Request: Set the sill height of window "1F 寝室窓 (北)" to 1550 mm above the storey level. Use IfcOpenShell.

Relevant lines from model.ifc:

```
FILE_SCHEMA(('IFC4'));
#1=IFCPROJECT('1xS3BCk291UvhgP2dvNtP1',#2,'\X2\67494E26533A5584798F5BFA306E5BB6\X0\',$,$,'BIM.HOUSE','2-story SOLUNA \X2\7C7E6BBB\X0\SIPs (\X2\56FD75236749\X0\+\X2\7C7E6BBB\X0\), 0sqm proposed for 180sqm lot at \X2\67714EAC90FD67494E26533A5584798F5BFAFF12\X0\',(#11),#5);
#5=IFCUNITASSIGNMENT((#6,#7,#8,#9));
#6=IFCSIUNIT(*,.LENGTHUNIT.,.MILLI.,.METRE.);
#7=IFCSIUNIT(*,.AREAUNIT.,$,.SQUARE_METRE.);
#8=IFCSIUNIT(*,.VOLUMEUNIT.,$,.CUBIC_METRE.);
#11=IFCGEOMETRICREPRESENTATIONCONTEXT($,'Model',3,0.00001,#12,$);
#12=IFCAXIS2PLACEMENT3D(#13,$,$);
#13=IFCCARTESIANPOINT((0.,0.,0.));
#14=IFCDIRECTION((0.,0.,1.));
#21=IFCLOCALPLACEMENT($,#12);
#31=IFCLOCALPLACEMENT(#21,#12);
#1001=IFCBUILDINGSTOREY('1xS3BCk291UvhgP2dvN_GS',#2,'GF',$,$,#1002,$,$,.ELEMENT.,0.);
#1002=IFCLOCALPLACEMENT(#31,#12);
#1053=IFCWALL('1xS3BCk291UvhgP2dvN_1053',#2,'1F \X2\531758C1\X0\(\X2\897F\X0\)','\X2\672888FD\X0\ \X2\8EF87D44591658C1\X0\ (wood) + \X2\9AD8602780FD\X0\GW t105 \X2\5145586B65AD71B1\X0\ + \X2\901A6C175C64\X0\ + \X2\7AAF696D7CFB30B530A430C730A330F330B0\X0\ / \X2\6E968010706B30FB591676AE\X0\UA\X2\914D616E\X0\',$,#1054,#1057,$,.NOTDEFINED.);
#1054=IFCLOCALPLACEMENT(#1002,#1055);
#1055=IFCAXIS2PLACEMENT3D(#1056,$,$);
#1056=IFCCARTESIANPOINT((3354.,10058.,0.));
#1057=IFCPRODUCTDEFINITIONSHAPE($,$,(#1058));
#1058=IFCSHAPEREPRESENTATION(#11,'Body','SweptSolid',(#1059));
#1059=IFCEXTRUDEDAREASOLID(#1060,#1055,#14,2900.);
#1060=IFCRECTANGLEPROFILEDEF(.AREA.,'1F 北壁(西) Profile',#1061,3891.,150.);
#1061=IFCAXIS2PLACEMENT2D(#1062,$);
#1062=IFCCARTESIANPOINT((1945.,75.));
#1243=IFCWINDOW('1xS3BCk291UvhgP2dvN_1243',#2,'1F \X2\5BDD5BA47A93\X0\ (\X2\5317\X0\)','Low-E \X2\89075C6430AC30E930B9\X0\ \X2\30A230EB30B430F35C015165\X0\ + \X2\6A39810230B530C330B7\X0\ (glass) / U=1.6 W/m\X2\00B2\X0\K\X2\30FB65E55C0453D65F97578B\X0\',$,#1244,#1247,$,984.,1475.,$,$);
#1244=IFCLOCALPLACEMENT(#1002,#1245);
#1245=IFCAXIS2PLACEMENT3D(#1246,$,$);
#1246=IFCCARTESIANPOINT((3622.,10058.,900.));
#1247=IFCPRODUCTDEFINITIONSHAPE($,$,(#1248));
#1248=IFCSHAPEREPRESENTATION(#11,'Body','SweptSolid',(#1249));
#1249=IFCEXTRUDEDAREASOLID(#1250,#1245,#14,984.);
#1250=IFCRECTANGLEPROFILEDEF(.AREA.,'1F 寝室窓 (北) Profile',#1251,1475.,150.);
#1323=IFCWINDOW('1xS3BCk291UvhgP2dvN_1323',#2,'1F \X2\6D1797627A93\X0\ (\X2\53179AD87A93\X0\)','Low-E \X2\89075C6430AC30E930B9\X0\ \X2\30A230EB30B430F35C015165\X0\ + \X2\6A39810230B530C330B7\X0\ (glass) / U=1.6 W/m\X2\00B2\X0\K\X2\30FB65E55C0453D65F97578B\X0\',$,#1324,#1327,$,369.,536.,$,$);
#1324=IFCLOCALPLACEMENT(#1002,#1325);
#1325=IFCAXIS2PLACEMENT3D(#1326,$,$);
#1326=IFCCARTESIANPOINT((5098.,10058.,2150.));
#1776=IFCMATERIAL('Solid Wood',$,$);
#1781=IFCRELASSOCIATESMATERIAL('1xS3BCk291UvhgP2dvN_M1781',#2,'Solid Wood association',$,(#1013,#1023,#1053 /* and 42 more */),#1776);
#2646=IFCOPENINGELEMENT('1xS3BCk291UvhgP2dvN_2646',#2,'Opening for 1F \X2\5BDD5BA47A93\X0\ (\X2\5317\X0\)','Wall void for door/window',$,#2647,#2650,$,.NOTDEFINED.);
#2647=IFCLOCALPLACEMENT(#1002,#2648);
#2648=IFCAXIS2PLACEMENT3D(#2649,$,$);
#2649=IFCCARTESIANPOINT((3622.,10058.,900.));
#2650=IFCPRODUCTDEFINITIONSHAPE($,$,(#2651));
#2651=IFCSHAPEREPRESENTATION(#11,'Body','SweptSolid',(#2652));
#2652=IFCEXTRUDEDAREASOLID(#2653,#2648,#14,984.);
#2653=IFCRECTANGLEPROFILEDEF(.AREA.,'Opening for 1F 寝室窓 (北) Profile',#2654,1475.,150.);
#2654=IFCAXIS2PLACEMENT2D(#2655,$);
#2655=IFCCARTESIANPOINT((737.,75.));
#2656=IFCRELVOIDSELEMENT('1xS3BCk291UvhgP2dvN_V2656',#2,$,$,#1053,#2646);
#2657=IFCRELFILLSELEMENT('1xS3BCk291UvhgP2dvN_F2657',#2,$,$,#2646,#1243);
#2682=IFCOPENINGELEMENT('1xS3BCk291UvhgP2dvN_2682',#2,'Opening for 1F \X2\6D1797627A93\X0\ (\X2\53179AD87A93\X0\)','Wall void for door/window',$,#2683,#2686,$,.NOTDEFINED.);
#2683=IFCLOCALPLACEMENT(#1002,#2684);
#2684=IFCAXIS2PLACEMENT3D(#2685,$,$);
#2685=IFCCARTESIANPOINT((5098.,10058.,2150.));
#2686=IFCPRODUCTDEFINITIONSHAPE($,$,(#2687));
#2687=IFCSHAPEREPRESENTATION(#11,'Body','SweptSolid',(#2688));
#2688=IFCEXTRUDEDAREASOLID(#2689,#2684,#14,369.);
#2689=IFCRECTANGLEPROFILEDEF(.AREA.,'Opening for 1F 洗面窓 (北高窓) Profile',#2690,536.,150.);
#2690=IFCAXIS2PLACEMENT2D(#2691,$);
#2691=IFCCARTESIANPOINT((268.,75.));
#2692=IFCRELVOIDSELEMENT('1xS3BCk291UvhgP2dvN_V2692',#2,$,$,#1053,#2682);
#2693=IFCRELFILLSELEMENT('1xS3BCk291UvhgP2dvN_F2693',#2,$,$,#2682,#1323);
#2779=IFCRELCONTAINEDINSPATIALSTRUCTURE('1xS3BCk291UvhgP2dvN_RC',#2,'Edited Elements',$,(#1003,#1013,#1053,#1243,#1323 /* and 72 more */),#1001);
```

```python
import numpy as np
import ifcopenshell
import ifcopenshell.api.geometry
import ifcopenshell.geom
import ifcopenshell.util.element
import ifcopenshell.util.placement
import ifcopenshell.util.shape
import ifcopenshell.util.unit

model = ifcopenshell.open("model.ifc")
unit_scale = ifcopenshell.util.unit.calculate_unit_scale(model)

window = model.by_guid("1xS3BCk291UvhgP2dvN_1243")
opening = window.FillsVoids[0].RelatingOpeningElement
storey = ifcopenshell.util.element.get_container(window, ifc_class="IfcBuildingStorey")
level = ifcopenshell.util.placement.get_local_placement(storey.ObjectPlacement)[2, 3]

# The opening's origin need not be at the sill, so measure its lowest point.
shape = ifcopenshell.geom.create_shape(ifcopenshell.geom.settings(), opening)
bottom = ifcopenshell.util.shape.get_shape_bottom_elevation(shape, shape.geometry) / unit_scale
dz = level + 1.55 / unit_scale - bottom

shift = np.array([0.0, 0.0, dz])
# The window is not placed relative to its opening, so move both.
for product in (opening, window):
    matrix = ifcopenshell.util.placement.get_local_placement(product.ObjectPlacement)
    matrix[:3, 3] += shift
    ifcopenshell.api.geometry.edit_object_placement(model, product=product, matrix=matrix, is_si=False)

print(f"moved by {dz * unit_scale:+.3f} m")

model.write("model_edited.ifc")
```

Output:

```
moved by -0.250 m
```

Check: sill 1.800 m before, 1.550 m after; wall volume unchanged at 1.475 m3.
